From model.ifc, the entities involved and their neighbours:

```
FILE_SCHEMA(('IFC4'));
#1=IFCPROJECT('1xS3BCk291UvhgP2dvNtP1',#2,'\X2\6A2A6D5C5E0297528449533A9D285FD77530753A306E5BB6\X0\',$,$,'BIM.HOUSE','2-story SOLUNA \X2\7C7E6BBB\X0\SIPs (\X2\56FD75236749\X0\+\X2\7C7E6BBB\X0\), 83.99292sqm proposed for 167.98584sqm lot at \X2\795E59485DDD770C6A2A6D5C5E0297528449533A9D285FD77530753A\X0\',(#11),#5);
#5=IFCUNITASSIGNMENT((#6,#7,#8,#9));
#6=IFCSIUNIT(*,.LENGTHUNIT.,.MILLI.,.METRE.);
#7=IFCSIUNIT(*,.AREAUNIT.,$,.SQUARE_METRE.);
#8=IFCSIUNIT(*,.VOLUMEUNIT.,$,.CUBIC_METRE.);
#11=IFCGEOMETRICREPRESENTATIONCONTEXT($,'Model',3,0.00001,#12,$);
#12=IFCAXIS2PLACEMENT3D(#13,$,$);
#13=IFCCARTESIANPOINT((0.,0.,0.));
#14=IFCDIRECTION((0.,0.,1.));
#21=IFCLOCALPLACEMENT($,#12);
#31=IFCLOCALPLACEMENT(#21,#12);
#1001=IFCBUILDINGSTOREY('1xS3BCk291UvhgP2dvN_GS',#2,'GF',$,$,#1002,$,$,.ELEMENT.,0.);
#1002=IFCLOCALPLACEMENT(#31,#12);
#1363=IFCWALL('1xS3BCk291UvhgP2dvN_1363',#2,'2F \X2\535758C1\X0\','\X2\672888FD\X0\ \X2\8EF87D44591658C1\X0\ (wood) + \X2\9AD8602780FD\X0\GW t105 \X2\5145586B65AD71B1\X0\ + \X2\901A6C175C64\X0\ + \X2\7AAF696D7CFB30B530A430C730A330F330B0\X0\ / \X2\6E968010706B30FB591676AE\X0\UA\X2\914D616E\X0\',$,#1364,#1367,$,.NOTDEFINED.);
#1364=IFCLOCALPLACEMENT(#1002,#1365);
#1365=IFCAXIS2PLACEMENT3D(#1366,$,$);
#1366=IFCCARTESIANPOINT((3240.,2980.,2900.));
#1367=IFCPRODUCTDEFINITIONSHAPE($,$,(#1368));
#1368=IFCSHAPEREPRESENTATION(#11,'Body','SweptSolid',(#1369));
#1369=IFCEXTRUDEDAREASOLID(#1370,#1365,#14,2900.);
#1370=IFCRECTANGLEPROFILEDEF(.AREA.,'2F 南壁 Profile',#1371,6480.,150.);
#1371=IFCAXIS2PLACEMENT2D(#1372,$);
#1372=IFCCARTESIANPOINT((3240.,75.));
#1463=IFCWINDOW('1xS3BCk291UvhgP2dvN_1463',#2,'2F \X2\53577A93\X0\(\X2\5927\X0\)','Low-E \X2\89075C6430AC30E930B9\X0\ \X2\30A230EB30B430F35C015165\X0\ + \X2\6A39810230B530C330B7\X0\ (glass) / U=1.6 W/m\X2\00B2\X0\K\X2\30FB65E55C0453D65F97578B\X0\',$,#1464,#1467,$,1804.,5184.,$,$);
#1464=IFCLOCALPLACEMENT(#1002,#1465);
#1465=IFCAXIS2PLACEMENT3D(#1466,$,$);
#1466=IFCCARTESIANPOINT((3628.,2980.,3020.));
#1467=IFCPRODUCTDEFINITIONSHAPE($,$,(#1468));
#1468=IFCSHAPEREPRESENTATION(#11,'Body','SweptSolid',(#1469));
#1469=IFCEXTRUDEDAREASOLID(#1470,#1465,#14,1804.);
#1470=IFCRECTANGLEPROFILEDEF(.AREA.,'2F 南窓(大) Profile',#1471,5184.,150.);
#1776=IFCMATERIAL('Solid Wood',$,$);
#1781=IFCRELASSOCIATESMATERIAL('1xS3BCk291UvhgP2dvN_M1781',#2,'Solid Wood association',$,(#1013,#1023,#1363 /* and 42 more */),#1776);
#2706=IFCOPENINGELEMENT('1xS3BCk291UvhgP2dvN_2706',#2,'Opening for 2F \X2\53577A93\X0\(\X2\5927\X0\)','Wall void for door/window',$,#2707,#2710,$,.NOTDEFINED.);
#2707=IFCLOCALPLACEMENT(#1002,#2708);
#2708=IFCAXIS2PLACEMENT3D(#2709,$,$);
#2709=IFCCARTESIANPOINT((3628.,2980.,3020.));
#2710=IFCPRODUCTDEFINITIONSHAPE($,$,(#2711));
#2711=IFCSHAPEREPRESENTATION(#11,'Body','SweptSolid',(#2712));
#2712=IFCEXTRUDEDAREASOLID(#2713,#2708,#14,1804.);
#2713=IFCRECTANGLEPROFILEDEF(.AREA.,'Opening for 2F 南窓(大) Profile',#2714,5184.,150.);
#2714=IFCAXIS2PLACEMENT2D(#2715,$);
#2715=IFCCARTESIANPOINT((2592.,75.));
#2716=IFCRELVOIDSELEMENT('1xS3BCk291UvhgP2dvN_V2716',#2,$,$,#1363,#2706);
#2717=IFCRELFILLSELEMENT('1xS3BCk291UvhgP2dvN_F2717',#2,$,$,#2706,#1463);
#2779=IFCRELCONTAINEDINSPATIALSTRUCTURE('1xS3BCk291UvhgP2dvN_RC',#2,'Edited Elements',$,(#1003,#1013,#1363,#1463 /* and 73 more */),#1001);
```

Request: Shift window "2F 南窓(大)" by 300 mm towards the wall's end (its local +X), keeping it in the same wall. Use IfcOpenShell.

```python
import ifcopenshell
import ifcopenshell.api.geometry
import ifcopenshell.util.placement

model = ifcopenshell.open("model.ifc")

window = model.by_guid("1xS3BCk291UvhgP2dvN_1463")
opening = window.FillsVoids[0].RelatingOpeningElement
wall = opening.VoidsElements[0].RelatingBuildingElement

wall_matrix = ifcopenshell.util.placement.get_local_placement(wall.ObjectPlacement)
shift = wall_matrix[:3, 0] * 300.0
before = ifcopenshell.util.placement.get_local_placement(window.ObjectPlacement)[:3, 3].copy()

# The window is not placed relative to its opening, so move both.
for product in (opening, window):
    matrix = ifcopenshell.util.placement.get_local_placement(product.ObjectPlacement)
    matrix[:3, 3] += shift
    ifcopenshell.api.geometry.edit_object_placement(model, product=product, matrix=matrix, is_si=False)

after = ifcopenshell.util.placement.get_local_placement(window.ObjectPlacement)[:3, 3]
print("window moved by", (after - before).round(3) + 0.0)

model.write("model_updated.ifc")
```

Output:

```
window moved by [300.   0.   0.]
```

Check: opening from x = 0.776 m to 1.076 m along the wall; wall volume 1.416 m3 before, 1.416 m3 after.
